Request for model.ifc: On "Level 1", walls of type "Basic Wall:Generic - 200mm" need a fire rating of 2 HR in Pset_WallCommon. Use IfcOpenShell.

First a look at what the model holds.

```python
import ifcopenshell
import ifcopenshell.util.element

model = ifcopenshell.open("model.ifc")
print(model.schema)
storey = next(s for s in model.by_type("IfcBuildingStorey") if s.Name == "Level 1")
walls = [e for e in ifcopenshell.util.element.get_decomposition(storey) if e.is_a("IfcWall")]
seen = {}
for e in walls:
    element_type = ifcopenshell.util.element.get_type(e)
    key = (element_type.Name if element_type != e and element_type else None, ifcopenshell.util.element.get_pset(e, "Pset_WallCommon", "FireRating"))
    seen[key] = seen.get(key, 0) + 1
for (name, value), count in sorted(seen.items(), key=str):
    print(count, "x", name, "|", value)
```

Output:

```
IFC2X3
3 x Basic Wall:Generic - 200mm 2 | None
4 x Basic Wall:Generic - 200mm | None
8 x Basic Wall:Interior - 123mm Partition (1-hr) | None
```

```python
import ifcopenshell
import ifcopenshell.api.pset
import ifcopenshell.util.element

model = ifcopenshell.open("model.ifc")

storey = next(s for s in model.by_type("IfcBuildingStorey") if s.Name == "Level 1")
walls = [e for e in ifcopenshell.util.element.get_decomposition(storey) if e.is_a("IfcWall")]

count = 0
for e in walls:
    element_type = ifcopenshell.util.element.get_type(e)
    if element_type in (None, e) or element_type.Name != "Basic Wall:Generic - 200mm":
        continue
    found = ifcopenshell.util.element.get_pset(e, "Pset_WallCommon", should_inherit=False)
    if found:
        pset = model.by_id(found["id"])
        if len(ifcopenshell.util.element.get_elements_by_pset(pset)) > 1:
            pset = ifcopenshell.api.pset.unshare_pset(model, products=[e], pset=pset)[0]
    else:
        pset = ifcopenshell.api.pset.add_pset(model, product=e, name="Pset_WallCommon")
    ifcopenshell.api.pset.edit_pset(model, pset=pset, properties={"FireRating": "2 HR"})
    count += 1

print(count, "walls updated")

model.write("model_rev.ifc")
```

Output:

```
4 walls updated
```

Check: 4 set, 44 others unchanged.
